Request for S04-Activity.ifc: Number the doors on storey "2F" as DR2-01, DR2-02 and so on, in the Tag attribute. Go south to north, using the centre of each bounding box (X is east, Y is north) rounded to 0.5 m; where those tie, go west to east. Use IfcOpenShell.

First a look at what the model holds.

```python
import ifcopenshell
import ifcopenshell.util.element
import ifcopenshell.util.placement

model = ifcopenshell.open("S04-Activity.ifc")
print(model.schema)
storey = next(s for s in model.by_type("IfcBuildingStorey") if s.Name == "2F")
doors = [e for e in ifcopenshell.util.element.get_decomposition(storey) if e.is_a("IfcDoor")]
for e in sorted(doors, key=lambda e: e.id()):
    origin = ifcopenshell.util.placement.get_local_placement(e.ObjectPlacement)[:3, 3]
    print(e.id(), e.Tag, e.Name, origin.round(2) + 0.0, sep=" | ")
```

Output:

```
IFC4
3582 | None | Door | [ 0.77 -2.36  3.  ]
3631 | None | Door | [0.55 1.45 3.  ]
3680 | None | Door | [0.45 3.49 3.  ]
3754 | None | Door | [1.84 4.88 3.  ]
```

```python
import ifcopenshell
import ifcopenshell.geom
import ifcopenshell.util.element
import ifcopenshell.util.shape

model = ifcopenshell.open("S04-Activity.ifc")
settings = ifcopenshell.geom.settings()
settings.set("use-world-coords", True)


def centre(element):
    shape = ifcopenshell.geom.create_shape(settings, element)
    return ifcopenshell.util.shape.get_bbox_centroid(shape.geometry)


storey = next(s for s in model.by_type("IfcBuildingStorey") if s.Name == "2F")
doors = [e for e in ifcopenshell.util.element.get_decomposition(storey) if e.is_a("IfcDoor")]

# Insertion points can sit at a corner or the storey origin, so sort by the geometry (in metres).
centres = {e: centre(e) for e in doors}
doors.sort(key=lambda e: (round(centres[e][1] / 0.5), centres[e][0]))

for i, e in enumerate(doors, start=1):
    number = f"DR2-{i:02d}"
    e.Tag = number
    print(e.id(), number)

model.write("S04-Activity_updated.ifc")
```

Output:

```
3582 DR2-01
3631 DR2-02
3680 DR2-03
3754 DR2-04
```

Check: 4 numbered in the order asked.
